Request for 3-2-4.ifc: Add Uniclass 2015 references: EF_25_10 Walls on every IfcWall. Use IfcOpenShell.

First a look at what the model holds.

```python
import ifcopenshell

model = ifcopenshell.open("3-2-4.ifc")
print(model.schema)
print("classifications:", [c.Name for c in model.by_type("IfcClassification")])
for ifc_class in ("IfcDoor", "IfcRoof", "IfcStair", "IfcWall", "IfcWindow"):
    print(ifc_class, len(model.by_type(ifc_class)))
```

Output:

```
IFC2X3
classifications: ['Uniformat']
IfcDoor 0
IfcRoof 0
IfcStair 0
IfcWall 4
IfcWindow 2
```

```python
import ifcopenshell
import ifcopenshell.api.classification

model = ifcopenshell.open("3-2-4.ifc")

# IFC2X3 requires Source and Edition and has no link from the project to the system.
system = model.create_entity("IfcClassification", Source="NBS", Edition="2015", Name="Uniclass 2015")

codes = {
    "IfcWall": ("EF_25_10", "Walls"),
}
for ifc_class, (code, name) in codes.items():
    products = model.by_type(ifc_class)
    ifcopenshell.api.classification.add_reference(
        model, products=products, classification=system, identification=code, name=name
    )
    print(code, len(products))

model.write("3-2-4_rev.ifc")
```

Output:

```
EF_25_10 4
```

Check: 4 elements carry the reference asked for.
